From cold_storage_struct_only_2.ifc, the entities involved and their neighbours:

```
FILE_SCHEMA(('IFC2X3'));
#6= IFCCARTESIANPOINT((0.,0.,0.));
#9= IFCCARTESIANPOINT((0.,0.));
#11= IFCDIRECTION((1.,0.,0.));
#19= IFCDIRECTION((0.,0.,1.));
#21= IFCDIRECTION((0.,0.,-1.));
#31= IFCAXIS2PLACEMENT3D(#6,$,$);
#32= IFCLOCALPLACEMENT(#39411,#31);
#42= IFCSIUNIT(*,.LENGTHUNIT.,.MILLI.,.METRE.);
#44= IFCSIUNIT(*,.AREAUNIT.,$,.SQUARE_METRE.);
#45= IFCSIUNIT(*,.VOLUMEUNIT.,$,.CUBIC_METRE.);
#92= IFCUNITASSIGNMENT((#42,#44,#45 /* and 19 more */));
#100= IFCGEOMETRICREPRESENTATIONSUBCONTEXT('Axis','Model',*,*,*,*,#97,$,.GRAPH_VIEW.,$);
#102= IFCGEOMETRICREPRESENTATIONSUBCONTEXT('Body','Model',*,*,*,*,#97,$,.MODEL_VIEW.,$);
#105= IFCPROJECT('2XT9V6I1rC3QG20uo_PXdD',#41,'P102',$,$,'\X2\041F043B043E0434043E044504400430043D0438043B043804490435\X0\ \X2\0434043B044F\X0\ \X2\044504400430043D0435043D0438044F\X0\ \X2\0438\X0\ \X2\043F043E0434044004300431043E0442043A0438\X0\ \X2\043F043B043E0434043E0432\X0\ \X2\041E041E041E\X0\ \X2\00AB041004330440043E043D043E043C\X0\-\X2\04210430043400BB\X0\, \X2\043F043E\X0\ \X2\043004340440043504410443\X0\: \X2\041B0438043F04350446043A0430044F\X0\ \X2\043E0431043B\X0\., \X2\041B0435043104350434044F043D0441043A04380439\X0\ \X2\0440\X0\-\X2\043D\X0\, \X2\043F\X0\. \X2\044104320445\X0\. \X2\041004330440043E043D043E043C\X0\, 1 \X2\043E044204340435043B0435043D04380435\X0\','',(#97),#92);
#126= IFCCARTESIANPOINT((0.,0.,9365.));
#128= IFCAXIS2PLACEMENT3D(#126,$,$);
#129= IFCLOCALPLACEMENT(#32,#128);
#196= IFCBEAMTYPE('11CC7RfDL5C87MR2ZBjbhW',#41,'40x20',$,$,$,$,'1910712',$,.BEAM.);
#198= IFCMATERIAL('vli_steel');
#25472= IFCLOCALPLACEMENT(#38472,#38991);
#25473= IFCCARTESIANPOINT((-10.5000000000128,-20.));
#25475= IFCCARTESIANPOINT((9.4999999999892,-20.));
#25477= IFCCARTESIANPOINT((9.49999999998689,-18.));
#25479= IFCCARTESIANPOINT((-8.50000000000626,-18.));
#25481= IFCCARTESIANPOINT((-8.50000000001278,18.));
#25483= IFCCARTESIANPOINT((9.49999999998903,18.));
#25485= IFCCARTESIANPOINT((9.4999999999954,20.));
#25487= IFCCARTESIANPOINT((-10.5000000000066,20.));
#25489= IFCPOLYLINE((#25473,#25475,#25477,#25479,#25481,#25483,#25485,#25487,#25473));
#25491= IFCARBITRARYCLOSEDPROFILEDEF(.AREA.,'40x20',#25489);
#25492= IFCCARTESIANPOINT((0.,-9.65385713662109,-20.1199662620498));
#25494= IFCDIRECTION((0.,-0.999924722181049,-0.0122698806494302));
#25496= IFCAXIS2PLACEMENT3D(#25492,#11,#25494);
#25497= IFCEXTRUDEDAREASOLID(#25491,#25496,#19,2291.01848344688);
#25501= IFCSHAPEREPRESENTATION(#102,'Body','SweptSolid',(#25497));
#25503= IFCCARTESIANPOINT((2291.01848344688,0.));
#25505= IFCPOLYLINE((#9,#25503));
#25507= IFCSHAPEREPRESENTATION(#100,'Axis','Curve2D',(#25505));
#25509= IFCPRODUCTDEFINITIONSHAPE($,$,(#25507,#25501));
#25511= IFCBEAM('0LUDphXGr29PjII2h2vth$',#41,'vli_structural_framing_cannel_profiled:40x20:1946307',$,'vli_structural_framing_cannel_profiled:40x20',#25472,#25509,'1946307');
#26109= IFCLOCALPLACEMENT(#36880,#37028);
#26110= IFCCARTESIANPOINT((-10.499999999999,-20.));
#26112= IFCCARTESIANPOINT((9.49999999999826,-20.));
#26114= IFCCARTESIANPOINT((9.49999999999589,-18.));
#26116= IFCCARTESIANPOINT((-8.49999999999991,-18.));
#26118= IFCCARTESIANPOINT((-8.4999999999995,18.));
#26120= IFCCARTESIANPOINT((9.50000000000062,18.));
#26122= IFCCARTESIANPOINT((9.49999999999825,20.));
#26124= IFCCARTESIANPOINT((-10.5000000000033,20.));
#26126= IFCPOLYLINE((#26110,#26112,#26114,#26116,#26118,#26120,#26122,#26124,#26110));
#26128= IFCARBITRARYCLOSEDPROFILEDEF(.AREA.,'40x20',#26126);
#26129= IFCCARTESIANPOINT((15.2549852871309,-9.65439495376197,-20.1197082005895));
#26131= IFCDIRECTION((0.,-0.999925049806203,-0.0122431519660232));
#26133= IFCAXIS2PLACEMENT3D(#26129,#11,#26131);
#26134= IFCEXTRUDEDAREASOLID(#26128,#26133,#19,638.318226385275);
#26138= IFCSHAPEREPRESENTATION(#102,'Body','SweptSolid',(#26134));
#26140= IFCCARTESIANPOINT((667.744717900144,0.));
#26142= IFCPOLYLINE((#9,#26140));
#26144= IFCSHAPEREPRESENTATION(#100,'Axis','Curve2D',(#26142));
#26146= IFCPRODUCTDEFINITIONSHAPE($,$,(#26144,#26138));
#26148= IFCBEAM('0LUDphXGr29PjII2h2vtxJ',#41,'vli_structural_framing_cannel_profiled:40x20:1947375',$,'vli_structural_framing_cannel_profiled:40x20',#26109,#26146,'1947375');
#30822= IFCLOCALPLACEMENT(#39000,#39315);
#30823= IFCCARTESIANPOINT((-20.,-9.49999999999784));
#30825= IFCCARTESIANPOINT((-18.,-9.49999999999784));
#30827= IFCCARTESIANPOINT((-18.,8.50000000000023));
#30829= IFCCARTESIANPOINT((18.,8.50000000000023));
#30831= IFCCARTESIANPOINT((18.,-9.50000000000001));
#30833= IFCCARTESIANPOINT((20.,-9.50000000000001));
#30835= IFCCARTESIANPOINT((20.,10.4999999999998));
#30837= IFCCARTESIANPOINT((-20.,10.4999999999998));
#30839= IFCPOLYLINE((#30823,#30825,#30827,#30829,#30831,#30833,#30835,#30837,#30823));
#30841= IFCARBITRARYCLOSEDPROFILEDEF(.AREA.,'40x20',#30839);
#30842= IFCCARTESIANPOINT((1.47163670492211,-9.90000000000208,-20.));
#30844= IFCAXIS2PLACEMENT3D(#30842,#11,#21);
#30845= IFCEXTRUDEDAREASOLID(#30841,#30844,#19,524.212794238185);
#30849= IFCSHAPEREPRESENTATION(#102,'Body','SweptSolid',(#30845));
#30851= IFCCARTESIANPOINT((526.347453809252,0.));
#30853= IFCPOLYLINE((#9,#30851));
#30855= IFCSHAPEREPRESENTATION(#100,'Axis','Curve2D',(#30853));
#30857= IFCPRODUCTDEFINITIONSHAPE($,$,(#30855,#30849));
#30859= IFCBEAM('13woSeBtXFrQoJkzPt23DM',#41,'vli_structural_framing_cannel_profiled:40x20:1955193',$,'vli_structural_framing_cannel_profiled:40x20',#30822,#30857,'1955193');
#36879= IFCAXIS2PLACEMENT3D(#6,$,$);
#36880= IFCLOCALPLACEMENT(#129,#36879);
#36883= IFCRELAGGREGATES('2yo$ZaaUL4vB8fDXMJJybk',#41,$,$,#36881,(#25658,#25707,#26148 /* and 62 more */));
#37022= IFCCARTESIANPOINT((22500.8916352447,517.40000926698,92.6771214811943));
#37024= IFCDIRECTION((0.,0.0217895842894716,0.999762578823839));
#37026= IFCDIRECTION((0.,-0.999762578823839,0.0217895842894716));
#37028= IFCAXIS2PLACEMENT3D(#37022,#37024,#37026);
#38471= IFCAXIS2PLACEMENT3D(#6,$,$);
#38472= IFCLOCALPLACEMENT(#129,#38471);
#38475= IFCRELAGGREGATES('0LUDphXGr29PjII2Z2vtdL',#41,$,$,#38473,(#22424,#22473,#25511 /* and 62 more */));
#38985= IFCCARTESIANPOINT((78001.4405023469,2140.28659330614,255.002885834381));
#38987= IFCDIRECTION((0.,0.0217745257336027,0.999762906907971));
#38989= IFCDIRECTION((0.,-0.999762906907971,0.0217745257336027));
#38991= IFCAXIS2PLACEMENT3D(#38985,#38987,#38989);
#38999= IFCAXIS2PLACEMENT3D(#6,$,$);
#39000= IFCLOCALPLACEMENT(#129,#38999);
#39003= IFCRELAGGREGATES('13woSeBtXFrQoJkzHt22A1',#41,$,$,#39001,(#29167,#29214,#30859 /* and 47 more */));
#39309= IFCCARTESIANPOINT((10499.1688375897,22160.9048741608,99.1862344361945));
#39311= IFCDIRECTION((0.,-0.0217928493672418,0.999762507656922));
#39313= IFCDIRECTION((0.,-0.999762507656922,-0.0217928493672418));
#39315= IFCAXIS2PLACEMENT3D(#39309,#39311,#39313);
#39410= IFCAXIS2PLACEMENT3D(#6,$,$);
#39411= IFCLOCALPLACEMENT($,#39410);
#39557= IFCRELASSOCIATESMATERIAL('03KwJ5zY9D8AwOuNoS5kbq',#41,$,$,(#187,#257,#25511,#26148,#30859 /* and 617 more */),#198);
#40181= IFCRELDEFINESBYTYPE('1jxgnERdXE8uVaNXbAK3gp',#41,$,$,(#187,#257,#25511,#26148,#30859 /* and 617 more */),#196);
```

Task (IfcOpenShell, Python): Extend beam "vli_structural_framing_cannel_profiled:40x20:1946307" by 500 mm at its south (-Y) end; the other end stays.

```python
import numpy as np
import ifcopenshell
import ifcopenshell.util.representation

model = ifcopenshell.open("cold_storage_struct_only_2.ifc")

member = model.by_guid("0LUDphXGr29PjII2h2vth$")
change = 500.0

# The extrusion runs towards the end named, so only its depth changes.
body = ifcopenshell.util.representation.get_representation(member, "Model", "Body")
solid = body.Items[0]
old_length = solid.Depth
solid.Depth += change

# Move the axis end point with it.
axis = next(r for r in member.Representation.Representations if r.RepresentationIdentifier == "Axis").Items[0]
start, end = (np.array(p.Coordinates) for p in axis.Points)
end = end + (end - start) / np.linalg.norm(end - start) * change
point = model.createIfcCartesianPoint(end.tolist())
axis.Points = [axis.Points[0], point]

print(f"length {old_length:g} -> {solid.Depth:g}")

model.write("cold_storage_struct_only_2_updated.ifc")
```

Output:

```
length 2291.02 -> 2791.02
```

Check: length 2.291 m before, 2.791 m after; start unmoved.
